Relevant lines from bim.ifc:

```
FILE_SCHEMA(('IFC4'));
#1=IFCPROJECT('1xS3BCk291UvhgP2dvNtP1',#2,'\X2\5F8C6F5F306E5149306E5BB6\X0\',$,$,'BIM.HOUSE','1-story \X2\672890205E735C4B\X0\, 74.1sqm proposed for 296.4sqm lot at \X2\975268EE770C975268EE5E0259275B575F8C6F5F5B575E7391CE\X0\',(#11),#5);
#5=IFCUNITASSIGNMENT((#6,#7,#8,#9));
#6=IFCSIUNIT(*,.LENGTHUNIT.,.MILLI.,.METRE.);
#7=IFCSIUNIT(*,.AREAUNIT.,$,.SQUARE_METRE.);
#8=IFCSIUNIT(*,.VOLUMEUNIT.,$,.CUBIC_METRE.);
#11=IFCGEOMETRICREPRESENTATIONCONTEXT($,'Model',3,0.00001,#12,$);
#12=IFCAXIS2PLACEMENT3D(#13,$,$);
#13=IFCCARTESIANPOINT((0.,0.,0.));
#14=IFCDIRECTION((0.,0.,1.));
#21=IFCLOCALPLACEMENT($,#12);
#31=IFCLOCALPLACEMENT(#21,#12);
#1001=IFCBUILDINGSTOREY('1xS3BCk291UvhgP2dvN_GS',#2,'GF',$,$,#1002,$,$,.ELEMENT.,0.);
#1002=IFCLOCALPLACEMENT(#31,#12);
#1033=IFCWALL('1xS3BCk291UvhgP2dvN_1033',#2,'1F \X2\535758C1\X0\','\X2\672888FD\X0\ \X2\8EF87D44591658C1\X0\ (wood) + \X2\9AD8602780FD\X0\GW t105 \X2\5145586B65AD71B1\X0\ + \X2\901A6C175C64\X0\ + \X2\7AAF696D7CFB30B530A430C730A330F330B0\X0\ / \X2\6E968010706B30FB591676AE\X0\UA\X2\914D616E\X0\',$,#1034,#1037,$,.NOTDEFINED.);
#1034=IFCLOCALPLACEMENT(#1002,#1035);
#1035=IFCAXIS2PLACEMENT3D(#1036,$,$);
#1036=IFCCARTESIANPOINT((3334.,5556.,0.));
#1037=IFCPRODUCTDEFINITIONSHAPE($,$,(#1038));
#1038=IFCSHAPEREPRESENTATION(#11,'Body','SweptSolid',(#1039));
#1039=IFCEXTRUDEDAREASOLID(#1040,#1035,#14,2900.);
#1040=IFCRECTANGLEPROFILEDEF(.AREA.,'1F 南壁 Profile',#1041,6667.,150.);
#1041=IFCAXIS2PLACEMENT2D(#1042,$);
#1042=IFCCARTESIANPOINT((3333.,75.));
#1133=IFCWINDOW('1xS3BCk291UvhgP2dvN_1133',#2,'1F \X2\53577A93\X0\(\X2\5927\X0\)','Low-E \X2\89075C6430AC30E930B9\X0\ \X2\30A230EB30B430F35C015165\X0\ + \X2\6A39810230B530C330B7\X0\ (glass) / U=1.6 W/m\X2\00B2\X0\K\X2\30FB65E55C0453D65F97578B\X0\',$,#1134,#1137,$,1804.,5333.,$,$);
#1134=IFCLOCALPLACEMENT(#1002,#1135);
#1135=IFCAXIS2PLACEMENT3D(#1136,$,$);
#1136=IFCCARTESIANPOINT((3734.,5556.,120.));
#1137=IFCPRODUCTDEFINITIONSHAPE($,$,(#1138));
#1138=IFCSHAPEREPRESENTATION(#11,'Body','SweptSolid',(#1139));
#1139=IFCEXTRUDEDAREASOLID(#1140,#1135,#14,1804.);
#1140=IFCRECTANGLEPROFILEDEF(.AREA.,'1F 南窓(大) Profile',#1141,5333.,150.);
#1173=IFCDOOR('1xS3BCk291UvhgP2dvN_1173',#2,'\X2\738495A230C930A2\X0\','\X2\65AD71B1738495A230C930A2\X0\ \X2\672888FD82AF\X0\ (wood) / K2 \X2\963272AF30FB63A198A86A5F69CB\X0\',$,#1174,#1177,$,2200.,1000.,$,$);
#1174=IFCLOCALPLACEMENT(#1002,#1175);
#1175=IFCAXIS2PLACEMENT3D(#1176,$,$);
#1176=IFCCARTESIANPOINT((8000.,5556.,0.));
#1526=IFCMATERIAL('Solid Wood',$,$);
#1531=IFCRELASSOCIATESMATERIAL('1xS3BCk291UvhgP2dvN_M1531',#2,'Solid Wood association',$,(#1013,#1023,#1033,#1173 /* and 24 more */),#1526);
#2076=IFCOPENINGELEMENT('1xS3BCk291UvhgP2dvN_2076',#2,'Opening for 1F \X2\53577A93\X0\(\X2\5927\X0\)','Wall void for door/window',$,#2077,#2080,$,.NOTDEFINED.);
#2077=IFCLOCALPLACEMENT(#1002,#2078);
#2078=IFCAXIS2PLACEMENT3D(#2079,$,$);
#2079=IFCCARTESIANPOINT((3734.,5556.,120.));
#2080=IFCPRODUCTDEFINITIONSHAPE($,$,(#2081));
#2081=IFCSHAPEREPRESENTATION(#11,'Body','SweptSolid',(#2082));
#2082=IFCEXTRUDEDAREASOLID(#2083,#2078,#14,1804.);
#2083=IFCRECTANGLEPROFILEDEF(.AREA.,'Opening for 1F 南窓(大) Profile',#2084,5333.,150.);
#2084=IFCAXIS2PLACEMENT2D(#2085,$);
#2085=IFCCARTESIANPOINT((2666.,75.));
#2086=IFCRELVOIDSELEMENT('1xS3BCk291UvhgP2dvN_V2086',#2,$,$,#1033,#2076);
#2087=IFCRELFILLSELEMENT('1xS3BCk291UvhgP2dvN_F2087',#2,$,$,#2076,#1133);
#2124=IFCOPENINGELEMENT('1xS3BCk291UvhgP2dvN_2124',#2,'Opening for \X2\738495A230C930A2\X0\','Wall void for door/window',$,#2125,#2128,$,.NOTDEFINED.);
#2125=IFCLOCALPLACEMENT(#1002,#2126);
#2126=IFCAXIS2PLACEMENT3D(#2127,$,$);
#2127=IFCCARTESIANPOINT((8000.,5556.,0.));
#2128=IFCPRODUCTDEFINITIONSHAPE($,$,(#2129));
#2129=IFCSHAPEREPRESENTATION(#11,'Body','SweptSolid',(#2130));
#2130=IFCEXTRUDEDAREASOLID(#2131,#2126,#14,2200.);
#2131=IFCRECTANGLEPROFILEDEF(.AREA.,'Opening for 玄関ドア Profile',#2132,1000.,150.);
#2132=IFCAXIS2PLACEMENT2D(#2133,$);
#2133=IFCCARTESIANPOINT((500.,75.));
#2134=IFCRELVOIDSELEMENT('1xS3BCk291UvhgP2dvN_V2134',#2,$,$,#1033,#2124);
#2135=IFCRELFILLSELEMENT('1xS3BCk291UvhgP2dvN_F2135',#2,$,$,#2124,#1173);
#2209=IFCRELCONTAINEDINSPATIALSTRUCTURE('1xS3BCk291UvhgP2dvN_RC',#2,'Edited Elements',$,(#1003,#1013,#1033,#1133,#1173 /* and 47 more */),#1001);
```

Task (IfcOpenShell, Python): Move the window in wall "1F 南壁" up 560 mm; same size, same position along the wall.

```python
import numpy as np
import ifcopenshell
import ifcopenshell.api.geometry
import ifcopenshell.util.placement
import ifcopenshell.util.unit

model = ifcopenshell.open("bim.ifc")
unit_scale = ifcopenshell.util.unit.calculate_unit_scale(model)

window = model.by_guid("1xS3BCk291UvhgP2dvN_1133")
opening = window.FillsVoids[0].RelatingOpeningElement
dz = 560.0

shift = np.array([0.0, 0.0, dz])
# The window is not placed relative to its opening, so move both.
for product in (opening, window):
    matrix = ifcopenshell.util.placement.get_local_placement(product.ObjectPlacement)
    matrix[:3, 3] += shift
    ifcopenshell.api.geometry.edit_object_placement(model, product=product, matrix=matrix, is_si=False)

print(f"moved by {dz * unit_scale:+.3f} m")

model.write("bim_v2.ifc")
```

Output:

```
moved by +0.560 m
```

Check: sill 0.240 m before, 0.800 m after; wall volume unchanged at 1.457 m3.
